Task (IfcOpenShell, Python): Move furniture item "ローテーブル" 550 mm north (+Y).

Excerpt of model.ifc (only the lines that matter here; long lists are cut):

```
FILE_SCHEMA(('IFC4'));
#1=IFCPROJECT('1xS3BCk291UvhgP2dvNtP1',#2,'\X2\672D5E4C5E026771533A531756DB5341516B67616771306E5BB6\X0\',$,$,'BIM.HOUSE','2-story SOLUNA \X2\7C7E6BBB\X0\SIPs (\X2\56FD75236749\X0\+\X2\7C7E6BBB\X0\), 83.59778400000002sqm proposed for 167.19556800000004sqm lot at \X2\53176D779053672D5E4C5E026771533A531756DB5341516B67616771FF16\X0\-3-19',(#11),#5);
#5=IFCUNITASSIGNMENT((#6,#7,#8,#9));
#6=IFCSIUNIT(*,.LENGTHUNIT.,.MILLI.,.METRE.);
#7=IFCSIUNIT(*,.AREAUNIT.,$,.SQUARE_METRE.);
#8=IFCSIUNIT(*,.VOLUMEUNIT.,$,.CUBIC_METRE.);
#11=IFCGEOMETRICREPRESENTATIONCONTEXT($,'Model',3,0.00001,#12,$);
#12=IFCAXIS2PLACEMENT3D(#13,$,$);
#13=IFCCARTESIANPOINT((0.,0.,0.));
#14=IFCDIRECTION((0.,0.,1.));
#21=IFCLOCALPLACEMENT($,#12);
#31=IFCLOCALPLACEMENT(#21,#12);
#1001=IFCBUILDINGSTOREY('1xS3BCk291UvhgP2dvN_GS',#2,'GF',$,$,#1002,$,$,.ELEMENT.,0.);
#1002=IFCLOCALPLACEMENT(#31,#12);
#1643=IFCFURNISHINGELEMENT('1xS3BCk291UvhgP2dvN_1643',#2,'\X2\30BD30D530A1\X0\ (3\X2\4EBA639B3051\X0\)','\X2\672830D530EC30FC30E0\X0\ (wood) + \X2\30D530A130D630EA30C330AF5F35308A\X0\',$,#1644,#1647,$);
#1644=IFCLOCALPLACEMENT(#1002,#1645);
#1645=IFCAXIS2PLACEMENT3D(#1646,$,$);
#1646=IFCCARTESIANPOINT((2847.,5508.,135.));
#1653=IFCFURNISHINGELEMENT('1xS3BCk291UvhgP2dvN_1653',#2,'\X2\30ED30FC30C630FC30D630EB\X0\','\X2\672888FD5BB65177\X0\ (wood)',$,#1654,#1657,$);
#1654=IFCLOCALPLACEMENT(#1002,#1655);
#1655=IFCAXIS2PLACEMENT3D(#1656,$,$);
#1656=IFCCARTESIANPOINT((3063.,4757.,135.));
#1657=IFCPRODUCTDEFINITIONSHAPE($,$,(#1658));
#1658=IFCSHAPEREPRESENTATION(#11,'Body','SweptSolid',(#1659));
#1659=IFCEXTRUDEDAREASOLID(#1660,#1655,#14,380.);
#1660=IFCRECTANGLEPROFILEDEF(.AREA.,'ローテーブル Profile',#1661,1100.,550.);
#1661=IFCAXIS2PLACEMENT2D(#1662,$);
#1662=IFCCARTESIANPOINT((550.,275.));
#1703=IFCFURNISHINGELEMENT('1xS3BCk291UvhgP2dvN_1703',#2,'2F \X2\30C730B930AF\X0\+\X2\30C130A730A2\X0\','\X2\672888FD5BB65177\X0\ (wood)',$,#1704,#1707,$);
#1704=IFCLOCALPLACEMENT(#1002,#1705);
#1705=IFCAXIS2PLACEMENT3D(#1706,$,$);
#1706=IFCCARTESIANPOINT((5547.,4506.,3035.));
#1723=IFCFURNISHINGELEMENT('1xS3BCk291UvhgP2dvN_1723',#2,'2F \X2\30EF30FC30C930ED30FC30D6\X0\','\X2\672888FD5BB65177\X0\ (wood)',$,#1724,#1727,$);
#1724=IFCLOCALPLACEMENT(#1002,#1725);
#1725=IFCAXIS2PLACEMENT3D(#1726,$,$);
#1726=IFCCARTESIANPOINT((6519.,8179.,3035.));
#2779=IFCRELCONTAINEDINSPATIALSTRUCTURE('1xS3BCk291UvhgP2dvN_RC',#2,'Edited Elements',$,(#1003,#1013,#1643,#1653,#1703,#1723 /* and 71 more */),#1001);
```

```python
import ifcopenshell
import ifcopenshell.api.geometry
import ifcopenshell.util.placement
import ifcopenshell.util.unit

model = ifcopenshell.open("model.ifc")
unit_scale = ifcopenshell.util.unit.calculate_unit_scale(model)

item = model.by_guid("1xS3BCk291UvhgP2dvN_1653")
matrix = ifcopenshell.util.placement.get_local_placement(item.ObjectPlacement)
matrix[1, 3] += 0.55 / unit_scale
ifcopenshell.api.geometry.edit_object_placement(model, product=item, matrix=matrix, is_si=False)

print(ifcopenshell.util.placement.get_local_placement(item.ObjectPlacement).round(3) + 0.0)

model.write("model_edited.ifc")
```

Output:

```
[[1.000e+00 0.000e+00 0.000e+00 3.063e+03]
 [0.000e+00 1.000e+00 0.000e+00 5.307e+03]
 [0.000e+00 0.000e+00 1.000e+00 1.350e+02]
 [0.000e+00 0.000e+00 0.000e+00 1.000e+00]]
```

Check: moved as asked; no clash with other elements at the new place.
